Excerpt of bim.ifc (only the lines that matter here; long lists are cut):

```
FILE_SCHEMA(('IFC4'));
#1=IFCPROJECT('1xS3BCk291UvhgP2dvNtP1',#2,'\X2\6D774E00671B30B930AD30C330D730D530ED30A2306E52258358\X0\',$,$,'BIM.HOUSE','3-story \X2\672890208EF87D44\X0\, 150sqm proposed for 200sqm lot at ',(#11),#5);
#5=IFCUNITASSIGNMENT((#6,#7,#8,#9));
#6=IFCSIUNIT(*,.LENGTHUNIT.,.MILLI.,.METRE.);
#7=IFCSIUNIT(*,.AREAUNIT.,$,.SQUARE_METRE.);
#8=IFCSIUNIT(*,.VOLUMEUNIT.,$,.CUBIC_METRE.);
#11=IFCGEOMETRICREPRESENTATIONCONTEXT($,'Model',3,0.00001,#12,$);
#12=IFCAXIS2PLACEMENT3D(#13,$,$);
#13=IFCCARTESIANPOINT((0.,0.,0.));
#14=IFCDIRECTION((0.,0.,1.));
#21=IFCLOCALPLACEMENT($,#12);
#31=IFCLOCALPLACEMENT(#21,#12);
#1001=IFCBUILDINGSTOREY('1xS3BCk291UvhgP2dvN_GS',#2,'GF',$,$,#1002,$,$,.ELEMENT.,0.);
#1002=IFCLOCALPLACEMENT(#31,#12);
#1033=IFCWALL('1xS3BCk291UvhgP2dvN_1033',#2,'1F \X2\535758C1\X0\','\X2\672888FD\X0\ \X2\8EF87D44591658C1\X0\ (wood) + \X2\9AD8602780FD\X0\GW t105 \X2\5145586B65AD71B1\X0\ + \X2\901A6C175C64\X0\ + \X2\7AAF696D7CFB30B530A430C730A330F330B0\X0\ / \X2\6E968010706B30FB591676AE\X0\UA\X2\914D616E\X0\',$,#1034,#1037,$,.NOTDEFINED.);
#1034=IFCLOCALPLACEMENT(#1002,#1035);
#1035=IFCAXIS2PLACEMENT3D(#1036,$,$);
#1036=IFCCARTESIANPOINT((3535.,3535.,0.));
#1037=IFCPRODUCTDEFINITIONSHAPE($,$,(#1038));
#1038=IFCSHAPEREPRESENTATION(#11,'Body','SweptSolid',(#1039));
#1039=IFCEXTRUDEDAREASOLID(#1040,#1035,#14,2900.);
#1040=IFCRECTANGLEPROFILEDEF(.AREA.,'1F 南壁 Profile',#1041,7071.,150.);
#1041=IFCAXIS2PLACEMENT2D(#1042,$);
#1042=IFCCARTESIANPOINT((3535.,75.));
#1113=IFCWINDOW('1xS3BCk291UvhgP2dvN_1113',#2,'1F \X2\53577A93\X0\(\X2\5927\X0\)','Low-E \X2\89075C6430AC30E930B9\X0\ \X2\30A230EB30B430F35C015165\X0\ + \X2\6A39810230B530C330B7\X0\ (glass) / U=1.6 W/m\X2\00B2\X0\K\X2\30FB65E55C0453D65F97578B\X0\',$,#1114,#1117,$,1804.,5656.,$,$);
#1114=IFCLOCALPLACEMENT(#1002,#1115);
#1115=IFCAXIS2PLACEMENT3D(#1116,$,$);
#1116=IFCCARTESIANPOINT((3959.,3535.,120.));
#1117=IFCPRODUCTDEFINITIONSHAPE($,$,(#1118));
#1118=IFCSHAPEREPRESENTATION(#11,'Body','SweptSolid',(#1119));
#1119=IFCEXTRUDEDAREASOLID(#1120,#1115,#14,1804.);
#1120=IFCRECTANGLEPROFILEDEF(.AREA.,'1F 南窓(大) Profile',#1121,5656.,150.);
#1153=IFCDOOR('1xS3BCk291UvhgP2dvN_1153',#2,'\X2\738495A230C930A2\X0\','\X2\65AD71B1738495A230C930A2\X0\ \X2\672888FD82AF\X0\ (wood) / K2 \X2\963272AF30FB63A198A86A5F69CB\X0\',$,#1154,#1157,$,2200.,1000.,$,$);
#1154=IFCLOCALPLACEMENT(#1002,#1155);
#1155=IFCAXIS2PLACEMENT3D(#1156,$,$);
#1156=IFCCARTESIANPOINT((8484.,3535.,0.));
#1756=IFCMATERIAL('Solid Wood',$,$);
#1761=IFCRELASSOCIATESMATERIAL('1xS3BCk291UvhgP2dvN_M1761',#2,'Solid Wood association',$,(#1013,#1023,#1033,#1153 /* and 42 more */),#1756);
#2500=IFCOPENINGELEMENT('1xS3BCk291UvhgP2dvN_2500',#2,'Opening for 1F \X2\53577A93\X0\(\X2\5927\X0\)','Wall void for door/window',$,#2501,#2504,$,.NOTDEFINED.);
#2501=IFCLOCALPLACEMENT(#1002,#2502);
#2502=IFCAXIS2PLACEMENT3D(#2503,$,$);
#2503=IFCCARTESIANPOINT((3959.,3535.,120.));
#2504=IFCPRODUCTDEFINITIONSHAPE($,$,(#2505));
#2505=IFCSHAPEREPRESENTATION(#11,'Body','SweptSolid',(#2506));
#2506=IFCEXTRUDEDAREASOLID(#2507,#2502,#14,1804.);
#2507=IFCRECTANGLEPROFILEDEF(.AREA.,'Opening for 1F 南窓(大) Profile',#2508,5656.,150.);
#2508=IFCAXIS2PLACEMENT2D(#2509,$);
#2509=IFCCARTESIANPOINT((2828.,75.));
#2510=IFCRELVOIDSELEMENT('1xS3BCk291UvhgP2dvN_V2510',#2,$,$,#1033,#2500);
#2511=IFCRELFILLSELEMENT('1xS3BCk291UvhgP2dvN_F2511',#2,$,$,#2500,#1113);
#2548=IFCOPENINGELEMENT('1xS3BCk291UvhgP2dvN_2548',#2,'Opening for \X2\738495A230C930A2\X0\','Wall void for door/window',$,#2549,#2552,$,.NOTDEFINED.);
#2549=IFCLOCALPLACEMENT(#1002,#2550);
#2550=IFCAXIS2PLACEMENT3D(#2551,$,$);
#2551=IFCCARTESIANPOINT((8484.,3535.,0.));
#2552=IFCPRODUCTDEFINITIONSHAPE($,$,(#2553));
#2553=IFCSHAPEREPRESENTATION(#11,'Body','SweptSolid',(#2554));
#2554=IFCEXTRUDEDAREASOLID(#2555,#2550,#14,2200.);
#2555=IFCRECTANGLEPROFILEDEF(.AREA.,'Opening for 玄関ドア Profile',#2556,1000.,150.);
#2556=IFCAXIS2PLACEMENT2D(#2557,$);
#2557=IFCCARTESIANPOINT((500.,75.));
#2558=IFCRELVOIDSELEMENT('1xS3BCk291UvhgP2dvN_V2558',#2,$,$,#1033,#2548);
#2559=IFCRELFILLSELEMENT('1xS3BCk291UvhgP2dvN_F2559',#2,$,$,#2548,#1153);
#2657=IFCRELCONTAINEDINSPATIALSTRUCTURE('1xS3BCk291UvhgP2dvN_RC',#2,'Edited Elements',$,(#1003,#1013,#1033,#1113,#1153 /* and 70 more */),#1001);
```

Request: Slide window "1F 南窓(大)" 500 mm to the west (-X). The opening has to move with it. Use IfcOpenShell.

```python
import ifcopenshell
import ifcopenshell.api.geometry
import ifcopenshell.util.placement
import ifcopenshell.util.unit

model = ifcopenshell.open("bim.ifc")
unit_scale = ifcopenshell.util.unit.calculate_unit_scale(model)

window = model.by_id(1113)
opening = window.FillsVoids[0].RelatingOpeningElement
wall = opening.VoidsElements[0].RelatingBuildingElement

wall_matrix = ifcopenshell.util.placement.get_local_placement(wall.ObjectPlacement)
shift = wall_matrix[:3, 0] * -0.5 / unit_scale
before = ifcopenshell.util.placement.get_local_placement(window.ObjectPlacement)[:3, 3].copy()

# The window is not placed relative to its opening, so move both.
for product in (opening, window):
    matrix = ifcopenshell.util.placement.get_local_placement(product.ObjectPlacement)
    matrix[:3, 3] += shift
    ifcopenshell.api.geometry.edit_object_placement(model, product=product, matrix=matrix, is_si=False)

after = ifcopenshell.util.placement.get_local_placement(window.ObjectPlacement)[:3, 3]
print("window moved by", (after - before).round(3) + 0.0)

model.write("bim_edited.ifc")
```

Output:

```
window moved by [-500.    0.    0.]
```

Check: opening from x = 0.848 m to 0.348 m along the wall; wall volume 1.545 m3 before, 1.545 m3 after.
